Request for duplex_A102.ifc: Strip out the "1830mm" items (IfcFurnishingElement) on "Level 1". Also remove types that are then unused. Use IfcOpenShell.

First a look at what the model holds.

```python
import ifcopenshell
import ifcopenshell.util.element

model = ifcopenshell.open("duplex_A102.ifc")
print(model.schema)
storey = next(s for s in model.by_type("IfcBuildingStorey") if s.Name == "Level 1")
furniture = [e for e in ifcopenshell.util.element.get_decomposition(storey) if e.is_a("IfcFurnishingElement")]
seen = {}
for e in furniture:
    element_type = ifcopenshell.util.element.get_type(e)
    name = element_type.Name if element_type not in (None, e) else None
    seen[name] = seen.get(name, 0) + 1
for name, count in sorted(seen.items(), key=str):
    print(count, "x", name)
```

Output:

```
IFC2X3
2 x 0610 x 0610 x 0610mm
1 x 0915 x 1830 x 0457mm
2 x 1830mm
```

```python
import ifcopenshell
import ifcopenshell.api.root
import ifcopenshell.util.element

model = ifcopenshell.open("duplex_A102.ifc")

storey = next(s for s in model.by_type("IfcBuildingStorey") if s.Name == "Level 1")
furniture = [e for e in ifcopenshell.util.element.get_decomposition(storey) if e.is_a("IfcFurnishingElement")]
targets = [e for e in furniture if (t := ifcopenshell.util.element.get_type(e)) not in (None, e) and t.Name == "1830mm"]
types = {ifcopenshell.util.element.get_type(e) for e in targets} - {None, *targets}

for e in targets:
    ifcopenshell.api.root.remove_product(model, product=e)
print(len(targets), "removed")

unused = [t for t in types if not ifcopenshell.util.element.get_types(t)]
for t in unused:
    ifcopenshell.api.root.remove_product(model, product=t)
print(len(unused), "unused types removed")

model.write("duplex_A102_edited.ifc")
```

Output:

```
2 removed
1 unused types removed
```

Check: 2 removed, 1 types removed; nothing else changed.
